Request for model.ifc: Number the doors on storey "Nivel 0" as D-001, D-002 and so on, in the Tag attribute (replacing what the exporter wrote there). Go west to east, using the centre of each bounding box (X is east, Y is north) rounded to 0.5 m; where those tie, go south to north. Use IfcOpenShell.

First a look at what the model holds.

```python
import ifcopenshell
import ifcopenshell.util.element
import ifcopenshell.util.placement

model = ifcopenshell.open("model.ifc")
print(model.schema)
storey = next(s for s in model.by_type("IfcBuildingStorey") if s.Name == "Nivel 0")
doors = [e for e in ifcopenshell.util.element.get_decomposition(storey) if e.is_a("IfcDoor")]
for e in sorted(doors, key=lambda e: e.id()):
    origin = ifcopenshell.util.placement.get_local_placement(e.ObjectPlacement)[:3, 3]
    print(e.id(), e.Tag, e.Name, origin.round(2) + 0.0, sep=" | ")
```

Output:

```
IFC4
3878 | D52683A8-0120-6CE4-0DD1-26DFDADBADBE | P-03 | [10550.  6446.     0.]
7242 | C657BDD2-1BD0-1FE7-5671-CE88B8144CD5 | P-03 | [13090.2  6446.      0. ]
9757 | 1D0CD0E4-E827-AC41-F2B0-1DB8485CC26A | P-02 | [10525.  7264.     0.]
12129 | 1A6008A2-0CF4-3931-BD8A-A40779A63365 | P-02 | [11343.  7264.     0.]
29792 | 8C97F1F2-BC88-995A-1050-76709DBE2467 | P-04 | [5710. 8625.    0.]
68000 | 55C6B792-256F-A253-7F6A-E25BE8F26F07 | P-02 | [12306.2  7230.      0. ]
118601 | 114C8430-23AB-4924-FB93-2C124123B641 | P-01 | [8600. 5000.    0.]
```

```python
import ifcopenshell
import ifcopenshell.geom
import ifcopenshell.util.element
import ifcopenshell.util.shape

model = ifcopenshell.open("model.ifc")
settings = ifcopenshell.geom.settings()
settings.set("use-world-coords", True)


def centre(element):
    shape = ifcopenshell.geom.create_shape(settings, element)
    return ifcopenshell.util.shape.get_bbox_centroid(shape.geometry)


storey = next(s for s in model.by_type("IfcBuildingStorey") if s.Name == "Nivel 0")
doors = [e for e in ifcopenshell.util.element.get_decomposition(storey) if e.is_a("IfcDoor")]

# Insertion points can sit at a corner or the storey origin, so sort by the geometry (in metres).
centres = {e: centre(e) for e in doors}
doors.sort(key=lambda e: (round(centres[e][0] / 0.5), centres[e][1]))

for i, e in enumerate(doors, start=1):
    number = f"D-0{i:02d}"
    e.Tag = number
    print(e.id(), number)

model.write("model-out.ifc")
```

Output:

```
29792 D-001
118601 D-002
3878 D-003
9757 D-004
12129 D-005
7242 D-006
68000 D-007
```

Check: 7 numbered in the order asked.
